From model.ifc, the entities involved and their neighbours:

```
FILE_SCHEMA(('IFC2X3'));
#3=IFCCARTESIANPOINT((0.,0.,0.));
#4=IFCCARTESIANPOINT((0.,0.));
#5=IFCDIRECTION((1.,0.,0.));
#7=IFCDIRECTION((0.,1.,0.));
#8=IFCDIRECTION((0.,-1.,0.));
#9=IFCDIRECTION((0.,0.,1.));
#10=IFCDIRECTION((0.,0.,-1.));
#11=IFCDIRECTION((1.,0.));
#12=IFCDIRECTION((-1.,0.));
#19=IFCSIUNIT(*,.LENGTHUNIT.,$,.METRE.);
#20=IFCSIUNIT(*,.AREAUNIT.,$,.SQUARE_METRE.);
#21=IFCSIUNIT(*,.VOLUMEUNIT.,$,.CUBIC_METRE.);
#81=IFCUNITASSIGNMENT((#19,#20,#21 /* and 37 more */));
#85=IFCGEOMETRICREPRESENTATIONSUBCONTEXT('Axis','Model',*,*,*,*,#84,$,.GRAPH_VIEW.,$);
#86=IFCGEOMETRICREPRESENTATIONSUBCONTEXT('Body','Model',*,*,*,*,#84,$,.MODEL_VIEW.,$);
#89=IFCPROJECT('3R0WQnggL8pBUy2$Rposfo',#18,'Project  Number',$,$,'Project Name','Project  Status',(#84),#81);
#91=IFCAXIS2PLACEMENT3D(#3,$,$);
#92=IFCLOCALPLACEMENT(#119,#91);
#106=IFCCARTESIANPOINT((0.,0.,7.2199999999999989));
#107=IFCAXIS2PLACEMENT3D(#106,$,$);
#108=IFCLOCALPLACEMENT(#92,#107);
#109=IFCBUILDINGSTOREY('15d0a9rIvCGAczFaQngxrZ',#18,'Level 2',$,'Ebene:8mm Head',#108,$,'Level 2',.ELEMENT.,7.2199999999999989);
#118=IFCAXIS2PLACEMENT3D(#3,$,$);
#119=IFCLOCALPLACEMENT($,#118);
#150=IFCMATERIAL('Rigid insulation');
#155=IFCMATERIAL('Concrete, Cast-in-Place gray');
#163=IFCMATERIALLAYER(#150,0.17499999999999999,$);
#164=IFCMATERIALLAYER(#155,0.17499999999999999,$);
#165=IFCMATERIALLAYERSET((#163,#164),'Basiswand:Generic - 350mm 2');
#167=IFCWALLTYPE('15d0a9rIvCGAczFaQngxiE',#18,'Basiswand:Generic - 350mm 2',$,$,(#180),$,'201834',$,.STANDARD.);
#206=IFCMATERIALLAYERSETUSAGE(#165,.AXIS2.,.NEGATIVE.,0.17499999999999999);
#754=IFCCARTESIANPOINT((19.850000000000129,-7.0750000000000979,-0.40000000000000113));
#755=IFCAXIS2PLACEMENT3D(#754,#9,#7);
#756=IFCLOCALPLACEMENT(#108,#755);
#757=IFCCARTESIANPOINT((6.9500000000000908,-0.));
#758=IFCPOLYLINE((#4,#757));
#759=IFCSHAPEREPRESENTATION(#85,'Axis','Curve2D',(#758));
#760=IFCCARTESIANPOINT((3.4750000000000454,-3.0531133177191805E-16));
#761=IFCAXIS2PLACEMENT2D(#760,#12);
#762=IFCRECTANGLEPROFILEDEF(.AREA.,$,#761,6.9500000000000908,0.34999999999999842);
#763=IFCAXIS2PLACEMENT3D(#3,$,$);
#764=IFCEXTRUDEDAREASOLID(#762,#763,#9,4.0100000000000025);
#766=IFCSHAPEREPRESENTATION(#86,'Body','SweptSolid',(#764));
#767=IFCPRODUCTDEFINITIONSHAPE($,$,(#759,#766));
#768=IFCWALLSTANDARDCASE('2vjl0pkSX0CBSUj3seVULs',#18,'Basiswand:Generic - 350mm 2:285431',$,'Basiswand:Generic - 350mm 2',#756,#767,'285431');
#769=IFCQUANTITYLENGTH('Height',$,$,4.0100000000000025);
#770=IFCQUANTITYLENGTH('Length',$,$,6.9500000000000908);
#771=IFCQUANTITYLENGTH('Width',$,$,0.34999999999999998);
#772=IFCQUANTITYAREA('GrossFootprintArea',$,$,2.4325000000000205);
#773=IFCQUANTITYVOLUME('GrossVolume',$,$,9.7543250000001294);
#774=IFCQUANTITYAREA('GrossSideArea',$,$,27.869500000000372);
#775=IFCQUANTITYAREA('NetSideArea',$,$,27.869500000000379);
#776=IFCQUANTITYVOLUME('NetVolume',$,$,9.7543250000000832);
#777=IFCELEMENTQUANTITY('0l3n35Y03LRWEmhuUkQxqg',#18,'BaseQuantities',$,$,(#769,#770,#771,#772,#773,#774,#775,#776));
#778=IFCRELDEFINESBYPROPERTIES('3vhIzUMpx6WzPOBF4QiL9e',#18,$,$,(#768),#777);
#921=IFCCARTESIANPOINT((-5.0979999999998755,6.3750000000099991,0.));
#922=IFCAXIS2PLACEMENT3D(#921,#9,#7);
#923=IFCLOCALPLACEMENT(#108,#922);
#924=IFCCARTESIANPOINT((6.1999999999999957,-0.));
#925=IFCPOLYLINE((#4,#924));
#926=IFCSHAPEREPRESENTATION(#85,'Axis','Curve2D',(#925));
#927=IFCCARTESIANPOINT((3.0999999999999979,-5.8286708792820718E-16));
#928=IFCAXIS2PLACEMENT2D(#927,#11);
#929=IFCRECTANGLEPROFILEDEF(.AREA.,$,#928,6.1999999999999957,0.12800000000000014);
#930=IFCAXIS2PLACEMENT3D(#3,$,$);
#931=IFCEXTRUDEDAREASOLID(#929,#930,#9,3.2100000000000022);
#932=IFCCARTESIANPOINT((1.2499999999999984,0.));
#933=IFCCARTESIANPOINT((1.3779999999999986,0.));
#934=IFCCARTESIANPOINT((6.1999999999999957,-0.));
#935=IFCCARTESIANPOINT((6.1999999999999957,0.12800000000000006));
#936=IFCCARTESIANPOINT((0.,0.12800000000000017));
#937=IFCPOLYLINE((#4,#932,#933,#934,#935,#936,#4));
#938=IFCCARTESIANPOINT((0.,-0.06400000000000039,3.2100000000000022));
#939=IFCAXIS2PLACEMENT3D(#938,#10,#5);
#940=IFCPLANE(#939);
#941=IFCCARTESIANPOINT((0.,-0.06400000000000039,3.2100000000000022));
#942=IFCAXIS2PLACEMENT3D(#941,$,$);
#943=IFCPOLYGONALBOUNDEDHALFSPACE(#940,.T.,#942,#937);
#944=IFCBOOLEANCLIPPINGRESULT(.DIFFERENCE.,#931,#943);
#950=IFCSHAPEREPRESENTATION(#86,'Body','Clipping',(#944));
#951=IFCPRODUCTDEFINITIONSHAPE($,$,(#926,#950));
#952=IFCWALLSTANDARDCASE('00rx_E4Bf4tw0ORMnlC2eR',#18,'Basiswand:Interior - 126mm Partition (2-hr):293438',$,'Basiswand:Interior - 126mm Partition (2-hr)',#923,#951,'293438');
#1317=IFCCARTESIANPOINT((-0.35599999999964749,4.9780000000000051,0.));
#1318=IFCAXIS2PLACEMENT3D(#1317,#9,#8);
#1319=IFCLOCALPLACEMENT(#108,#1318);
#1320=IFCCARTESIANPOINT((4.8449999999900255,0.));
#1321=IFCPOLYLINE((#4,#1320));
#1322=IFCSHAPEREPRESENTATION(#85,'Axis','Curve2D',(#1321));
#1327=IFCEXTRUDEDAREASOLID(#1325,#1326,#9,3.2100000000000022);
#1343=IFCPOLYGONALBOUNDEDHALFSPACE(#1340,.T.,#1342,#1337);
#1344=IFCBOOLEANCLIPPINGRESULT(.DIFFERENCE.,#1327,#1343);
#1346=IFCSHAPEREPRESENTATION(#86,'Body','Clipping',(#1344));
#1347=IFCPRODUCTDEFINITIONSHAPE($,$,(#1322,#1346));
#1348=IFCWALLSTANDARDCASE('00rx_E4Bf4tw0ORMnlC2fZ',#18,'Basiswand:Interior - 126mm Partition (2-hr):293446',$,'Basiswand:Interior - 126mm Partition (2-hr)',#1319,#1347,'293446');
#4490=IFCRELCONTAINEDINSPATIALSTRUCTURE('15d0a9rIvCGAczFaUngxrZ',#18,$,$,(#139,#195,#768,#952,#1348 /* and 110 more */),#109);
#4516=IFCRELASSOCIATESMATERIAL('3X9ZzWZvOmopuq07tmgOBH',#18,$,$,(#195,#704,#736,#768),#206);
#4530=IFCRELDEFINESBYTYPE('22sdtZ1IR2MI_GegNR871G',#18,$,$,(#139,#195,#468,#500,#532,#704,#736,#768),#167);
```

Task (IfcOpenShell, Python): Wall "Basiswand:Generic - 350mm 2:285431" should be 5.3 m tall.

```python
import ifcopenshell
import ifcopenshell.api.pset
import ifcopenshell.geom
import ifcopenshell.util.element
import ifcopenshell.util.representation
import ifcopenshell.util.shape
import ifcopenshell.util.unit

model = ifcopenshell.open("model.ifc")
unit_scale = ifcopenshell.util.unit.calculate_unit_scale(model)
area_scale = ifcopenshell.util.unit.calculate_unit_scale(model, "AREAUNIT")
volume_scale = ifcopenshell.util.unit.calculate_unit_scale(model, "VOLUMEUNIT")
settings = ifcopenshell.geom.settings()


def volume(element):
    """Net volume in cubic metres, openings subtracted."""
    shape = ifcopenshell.geom.create_shape(settings, element)
    return ifcopenshell.util.shape.get_volume(shape.geometry)


wall = model.by_id(768)
before = volume(wall)

body = ifcopenshell.util.representation.get_representation(wall, "Model", "Body")
solid = body.Items[0]
old_height = solid.Depth
solid.Depth = 5.3 / unit_scale
after = volume(wall)
thickness = 0.35  # wall thickness in metres

# Update the stored height, areas and volumes.
qto = model.by_id(ifcopenshell.util.element.get_pset(wall, "BaseQuantities", should_inherit=False)["id"])
ifcopenshell.api.pset.edit_qto(model, qto=qto, properties={
    "Height": solid.Depth,
    "GrossVolume": ifcopenshell.util.element.get_pset(wall, "BaseQuantities", "GrossVolume") * solid.Depth / old_height,
    "GrossSideArea": ifcopenshell.util.element.get_pset(wall, "BaseQuantities", "GrossSideArea") * solid.Depth / old_height,
    "NetSideArea": after / thickness / area_scale,
    "NetVolume": after / volume_scale,
})

print(f"height {old_height:g} -> {solid.Depth:g}, volume {before:.3f} -> {after:.3f} m3")

model.write("model_rev.ifc")
```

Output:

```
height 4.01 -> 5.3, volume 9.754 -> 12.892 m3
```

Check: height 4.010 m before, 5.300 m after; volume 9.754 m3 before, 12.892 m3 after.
